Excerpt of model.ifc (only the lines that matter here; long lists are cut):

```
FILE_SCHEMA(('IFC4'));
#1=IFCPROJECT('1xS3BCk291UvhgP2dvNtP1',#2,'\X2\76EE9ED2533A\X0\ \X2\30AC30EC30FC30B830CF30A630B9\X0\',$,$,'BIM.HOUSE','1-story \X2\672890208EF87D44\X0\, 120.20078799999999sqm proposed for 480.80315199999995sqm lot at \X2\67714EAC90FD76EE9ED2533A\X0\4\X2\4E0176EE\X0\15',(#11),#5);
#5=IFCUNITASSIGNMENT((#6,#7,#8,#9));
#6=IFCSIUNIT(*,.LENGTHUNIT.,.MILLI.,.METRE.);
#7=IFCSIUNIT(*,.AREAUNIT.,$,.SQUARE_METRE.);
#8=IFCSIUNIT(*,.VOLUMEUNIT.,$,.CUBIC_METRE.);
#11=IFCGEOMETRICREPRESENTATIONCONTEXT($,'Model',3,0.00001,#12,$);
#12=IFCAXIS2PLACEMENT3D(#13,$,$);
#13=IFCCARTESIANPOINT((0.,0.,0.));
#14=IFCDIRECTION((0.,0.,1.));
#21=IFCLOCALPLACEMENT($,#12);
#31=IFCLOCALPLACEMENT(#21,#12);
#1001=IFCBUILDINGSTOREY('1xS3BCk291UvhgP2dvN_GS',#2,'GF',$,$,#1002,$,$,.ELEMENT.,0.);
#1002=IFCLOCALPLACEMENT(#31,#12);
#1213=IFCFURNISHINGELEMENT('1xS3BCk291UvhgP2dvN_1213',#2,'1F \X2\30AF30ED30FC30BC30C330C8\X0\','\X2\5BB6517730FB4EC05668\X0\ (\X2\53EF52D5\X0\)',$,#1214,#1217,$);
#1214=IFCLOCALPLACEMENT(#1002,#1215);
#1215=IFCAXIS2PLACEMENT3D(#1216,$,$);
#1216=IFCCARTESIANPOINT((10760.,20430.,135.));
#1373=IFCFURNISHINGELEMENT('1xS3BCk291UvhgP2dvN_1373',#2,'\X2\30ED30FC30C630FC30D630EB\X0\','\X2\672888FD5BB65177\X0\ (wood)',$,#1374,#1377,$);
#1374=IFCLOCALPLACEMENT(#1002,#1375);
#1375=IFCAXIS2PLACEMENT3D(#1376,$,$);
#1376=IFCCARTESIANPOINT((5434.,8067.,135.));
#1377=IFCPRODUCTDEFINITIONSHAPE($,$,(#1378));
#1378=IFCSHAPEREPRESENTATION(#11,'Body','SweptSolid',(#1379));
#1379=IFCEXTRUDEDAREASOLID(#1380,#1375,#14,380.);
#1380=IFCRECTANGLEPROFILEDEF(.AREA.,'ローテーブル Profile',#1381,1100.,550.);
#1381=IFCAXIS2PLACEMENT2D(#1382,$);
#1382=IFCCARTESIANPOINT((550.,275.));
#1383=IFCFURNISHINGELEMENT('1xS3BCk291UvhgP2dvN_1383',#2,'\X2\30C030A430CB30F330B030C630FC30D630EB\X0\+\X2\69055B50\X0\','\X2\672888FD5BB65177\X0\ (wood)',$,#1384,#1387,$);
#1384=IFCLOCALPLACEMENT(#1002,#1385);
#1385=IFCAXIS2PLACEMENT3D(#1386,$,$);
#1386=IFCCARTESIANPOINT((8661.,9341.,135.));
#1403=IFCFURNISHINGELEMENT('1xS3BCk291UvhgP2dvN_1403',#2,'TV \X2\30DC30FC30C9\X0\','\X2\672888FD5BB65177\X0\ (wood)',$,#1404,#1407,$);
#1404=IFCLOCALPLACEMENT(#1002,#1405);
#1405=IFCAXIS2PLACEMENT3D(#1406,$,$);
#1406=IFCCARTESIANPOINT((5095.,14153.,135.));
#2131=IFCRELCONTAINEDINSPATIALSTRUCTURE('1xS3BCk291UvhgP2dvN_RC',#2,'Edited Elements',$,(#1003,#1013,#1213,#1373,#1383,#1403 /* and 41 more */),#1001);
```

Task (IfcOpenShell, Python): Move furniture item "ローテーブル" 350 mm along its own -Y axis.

```python
import ifcopenshell
import ifcopenshell.api.geometry
import ifcopenshell.util.placement

model = ifcopenshell.open("model.ifc")

item = model.by_guid("1xS3BCk291UvhgP2dvN_1373")
matrix = ifcopenshell.util.placement.get_local_placement(item.ObjectPlacement)
matrix[:3, 3] -= matrix[:3, 1] * 350.0
ifcopenshell.api.geometry.edit_object_placement(model, product=item, matrix=matrix, is_si=False)

print(ifcopenshell.util.placement.get_local_placement(item.ObjectPlacement).round(3) + 0.0)

model.write("model-out.ifc")
```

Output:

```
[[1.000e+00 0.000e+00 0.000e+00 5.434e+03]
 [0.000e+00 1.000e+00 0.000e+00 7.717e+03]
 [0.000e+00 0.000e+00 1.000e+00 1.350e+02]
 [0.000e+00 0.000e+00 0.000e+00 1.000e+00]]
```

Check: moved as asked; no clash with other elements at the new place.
